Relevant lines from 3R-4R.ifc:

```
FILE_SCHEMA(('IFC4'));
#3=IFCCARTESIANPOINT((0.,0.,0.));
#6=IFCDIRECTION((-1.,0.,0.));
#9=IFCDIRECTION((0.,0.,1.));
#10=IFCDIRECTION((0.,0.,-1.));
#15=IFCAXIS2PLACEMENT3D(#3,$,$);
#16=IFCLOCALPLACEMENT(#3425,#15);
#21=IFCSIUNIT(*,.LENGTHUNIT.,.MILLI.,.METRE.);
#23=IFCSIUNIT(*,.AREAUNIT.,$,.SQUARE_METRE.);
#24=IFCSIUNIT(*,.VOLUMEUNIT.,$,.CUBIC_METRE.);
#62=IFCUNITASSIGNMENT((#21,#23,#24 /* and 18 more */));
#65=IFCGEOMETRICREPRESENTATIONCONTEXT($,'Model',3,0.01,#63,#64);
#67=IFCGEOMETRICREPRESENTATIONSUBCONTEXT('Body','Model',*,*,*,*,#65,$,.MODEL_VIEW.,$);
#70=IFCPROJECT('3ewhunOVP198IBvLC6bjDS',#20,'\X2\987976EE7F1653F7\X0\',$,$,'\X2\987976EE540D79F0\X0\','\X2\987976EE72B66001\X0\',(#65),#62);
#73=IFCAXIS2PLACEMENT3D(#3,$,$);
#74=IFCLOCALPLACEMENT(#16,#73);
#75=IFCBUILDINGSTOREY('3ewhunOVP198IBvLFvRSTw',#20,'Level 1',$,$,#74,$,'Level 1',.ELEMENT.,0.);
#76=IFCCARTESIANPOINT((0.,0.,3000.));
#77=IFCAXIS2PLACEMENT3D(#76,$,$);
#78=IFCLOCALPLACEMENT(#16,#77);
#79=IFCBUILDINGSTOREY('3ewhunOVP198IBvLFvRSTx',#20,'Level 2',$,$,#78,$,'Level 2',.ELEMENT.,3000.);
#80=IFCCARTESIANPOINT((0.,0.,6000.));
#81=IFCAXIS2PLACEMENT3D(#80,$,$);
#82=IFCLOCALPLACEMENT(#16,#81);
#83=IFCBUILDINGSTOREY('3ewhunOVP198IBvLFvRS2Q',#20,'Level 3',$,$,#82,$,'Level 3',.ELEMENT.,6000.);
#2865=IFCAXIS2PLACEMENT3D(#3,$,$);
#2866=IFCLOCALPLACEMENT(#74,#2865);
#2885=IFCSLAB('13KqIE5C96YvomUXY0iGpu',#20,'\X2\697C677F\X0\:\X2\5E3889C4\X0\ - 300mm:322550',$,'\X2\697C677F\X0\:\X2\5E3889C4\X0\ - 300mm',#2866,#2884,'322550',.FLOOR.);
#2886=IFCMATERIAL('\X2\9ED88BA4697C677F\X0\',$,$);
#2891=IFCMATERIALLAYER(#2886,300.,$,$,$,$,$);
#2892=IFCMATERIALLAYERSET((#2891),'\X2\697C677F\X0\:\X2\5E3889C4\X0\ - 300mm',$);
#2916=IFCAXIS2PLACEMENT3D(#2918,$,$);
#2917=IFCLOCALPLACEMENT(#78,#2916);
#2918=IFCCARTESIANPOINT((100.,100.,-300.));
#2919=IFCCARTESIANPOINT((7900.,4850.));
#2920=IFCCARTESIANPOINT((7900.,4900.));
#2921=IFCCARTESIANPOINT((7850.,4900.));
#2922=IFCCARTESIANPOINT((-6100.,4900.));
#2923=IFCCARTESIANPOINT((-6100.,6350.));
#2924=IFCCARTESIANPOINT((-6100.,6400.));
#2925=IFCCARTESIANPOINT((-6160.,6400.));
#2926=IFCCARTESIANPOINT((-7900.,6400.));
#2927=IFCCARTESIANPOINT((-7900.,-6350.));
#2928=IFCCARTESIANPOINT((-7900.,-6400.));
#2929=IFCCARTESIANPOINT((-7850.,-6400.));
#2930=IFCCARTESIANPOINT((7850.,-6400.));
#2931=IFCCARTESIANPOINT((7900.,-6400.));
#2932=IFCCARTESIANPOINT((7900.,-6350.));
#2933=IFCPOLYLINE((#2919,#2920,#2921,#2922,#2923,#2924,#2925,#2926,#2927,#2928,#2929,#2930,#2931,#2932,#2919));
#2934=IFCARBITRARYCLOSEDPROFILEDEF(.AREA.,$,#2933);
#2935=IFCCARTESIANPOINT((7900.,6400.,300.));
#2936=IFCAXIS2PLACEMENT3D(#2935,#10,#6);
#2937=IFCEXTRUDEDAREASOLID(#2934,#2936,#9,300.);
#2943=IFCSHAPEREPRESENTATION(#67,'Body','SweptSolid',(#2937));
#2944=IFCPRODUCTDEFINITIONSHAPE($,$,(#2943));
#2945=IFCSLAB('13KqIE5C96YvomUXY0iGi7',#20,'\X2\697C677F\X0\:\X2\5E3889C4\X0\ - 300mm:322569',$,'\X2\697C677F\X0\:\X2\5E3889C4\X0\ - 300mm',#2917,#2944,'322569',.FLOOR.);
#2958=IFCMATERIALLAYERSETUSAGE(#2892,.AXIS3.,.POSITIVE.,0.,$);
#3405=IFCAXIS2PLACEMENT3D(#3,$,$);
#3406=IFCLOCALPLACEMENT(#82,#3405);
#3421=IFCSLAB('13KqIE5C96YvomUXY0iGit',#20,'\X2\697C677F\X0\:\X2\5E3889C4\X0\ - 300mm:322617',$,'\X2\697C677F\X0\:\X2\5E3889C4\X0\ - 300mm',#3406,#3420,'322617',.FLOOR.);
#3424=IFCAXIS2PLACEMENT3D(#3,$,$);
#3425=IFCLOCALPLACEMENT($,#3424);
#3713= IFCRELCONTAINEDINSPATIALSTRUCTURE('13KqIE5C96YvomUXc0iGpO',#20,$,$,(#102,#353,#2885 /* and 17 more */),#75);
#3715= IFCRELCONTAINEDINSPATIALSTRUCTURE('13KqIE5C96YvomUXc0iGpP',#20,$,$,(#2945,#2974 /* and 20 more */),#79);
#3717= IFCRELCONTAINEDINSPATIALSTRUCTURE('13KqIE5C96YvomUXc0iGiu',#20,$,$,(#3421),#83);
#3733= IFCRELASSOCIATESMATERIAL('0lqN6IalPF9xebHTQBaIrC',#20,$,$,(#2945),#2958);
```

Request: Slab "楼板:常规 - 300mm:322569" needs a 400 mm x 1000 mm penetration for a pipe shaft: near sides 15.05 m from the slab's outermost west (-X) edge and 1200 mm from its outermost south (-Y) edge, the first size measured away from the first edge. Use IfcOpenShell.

```python
import numpy as np
import ifcopenshell
import ifcopenshell.api.feature
import ifcopenshell.api.geometry
import ifcopenshell.api.root
import ifcopenshell.geom
import ifcopenshell.util.placement
import ifcopenshell.util.representation
import ifcopenshell.util.shape
import ifcopenshell.util.unit

model = ifcopenshell.open("3R-4R.ifc")
unit_scale = ifcopenshell.util.unit.calculate_unit_scale(model)
settings = ifcopenshell.geom.settings()


def volume(element):
    """Net volume in cubic metres, openings subtracted."""
    shape = ifcopenshell.geom.create_shape(settings, element)
    return ifcopenshell.util.shape.get_volume(shape.geometry)


slab = model.by_guid("13KqIE5C96YvomUXY0iGi7")
before = volume(slab)

# Extent in the slab's own axes, in metres. The edges named are its -X and -Y sides.
slab_shape = ifcopenshell.geom.create_shape(settings, slab)
vertices = ifcopenshell.util.shape.get_vertices(slab_shape.geometry)
x_min, y_min, bottom = vertices.min(axis=0)
top = vertices[:, 2].max()

opening = ifcopenshell.api.root.create_entity(model, ifc_class="IfcOpeningElement", name="Pipe shaft opening", predefined_type="OPENING")
context = ifcopenshell.util.representation.get_context(model, "Model", "Body", "MODEL_VIEW")
width, depth = 0.4, 1
outline = [(0.0, 0.0), (width, 0.0), (width, depth), (0.0, depth), (0.0, 0.0)]
# Overshoot both faces by 50 mm so the cut is clean.
shape = ifcopenshell.api.geometry.add_slab_representation(
    model, context=context, depth=top - bottom + 0.1, polyline=outline
)
ifcopenshell.api.geometry.assign_representation(model, product=opening, representation=shape)

matrix = ifcopenshell.util.placement.get_local_placement(slab.ObjectPlacement)
matrix[:, 3] = matrix @ np.append(np.array([x_min + 15.05, y_min + 1.2, bottom - 0.05]) / unit_scale, 1.0)
ifcopenshell.api.geometry.edit_object_placement(model, product=opening, matrix=matrix, is_si=False)
ifcopenshell.api.feature.add_feature(model, feature=opening, element=slab)

after = volume(slab)

print(f"slab volume {before:.3f} -> {after:.3f} m3")

model.write("3R-4R_edited.ifc")
```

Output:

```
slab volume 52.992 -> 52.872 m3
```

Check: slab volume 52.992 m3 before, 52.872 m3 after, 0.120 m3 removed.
